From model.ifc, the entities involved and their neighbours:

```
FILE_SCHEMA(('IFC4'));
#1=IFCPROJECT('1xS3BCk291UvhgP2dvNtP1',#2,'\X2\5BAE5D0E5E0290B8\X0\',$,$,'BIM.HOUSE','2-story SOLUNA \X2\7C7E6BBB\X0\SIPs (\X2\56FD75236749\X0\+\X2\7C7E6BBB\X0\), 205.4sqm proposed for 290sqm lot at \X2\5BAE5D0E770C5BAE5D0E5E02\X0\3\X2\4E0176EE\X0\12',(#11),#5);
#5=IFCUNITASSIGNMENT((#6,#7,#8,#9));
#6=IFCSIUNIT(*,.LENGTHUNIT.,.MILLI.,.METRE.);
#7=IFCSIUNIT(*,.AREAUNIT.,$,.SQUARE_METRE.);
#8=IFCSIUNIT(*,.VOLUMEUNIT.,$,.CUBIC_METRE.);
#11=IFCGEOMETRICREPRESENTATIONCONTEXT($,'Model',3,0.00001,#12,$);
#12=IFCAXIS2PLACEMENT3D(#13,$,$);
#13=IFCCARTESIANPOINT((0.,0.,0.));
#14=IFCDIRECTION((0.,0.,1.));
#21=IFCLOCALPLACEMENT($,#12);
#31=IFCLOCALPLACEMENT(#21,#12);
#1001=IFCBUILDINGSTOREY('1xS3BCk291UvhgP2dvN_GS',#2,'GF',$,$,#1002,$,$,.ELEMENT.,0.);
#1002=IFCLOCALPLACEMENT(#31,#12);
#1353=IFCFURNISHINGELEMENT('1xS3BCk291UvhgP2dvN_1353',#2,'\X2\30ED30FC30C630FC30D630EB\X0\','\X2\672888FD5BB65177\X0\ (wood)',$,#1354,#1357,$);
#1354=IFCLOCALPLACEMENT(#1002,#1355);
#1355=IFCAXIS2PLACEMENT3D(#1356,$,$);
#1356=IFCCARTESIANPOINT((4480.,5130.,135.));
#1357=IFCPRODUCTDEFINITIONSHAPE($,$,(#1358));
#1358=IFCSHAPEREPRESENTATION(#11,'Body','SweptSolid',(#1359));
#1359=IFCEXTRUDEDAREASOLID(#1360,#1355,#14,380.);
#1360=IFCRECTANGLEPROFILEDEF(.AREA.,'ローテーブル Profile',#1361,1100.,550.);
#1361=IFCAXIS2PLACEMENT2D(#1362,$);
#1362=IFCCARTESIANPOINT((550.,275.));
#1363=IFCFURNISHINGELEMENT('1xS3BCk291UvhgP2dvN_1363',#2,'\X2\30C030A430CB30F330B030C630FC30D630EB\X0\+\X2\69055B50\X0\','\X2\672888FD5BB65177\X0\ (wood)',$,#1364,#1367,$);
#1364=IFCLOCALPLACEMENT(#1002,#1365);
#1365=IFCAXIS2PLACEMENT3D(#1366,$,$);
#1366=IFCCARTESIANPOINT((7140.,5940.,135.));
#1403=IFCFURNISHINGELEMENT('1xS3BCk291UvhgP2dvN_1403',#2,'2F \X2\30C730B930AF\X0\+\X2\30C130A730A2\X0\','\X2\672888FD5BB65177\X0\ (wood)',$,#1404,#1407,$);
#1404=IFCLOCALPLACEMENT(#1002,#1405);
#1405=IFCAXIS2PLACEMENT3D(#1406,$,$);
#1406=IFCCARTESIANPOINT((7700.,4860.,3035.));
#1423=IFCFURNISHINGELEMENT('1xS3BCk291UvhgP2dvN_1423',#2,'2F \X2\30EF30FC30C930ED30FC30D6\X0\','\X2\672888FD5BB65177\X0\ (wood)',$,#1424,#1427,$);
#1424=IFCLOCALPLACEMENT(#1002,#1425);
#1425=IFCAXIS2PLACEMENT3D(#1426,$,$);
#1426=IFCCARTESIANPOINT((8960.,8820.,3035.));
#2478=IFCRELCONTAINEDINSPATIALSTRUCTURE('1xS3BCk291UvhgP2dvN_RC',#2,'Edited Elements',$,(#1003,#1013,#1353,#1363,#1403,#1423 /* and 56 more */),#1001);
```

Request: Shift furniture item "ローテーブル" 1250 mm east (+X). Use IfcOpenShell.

```python
import ifcopenshell
import ifcopenshell.api.geometry
import ifcopenshell.util.placement
import ifcopenshell.util.unit

model = ifcopenshell.open("model.ifc")
unit_scale = ifcopenshell.util.unit.calculate_unit_scale(model)

item = model.by_guid("1xS3BCk291UvhgP2dvN_1353")
matrix = ifcopenshell.util.placement.get_local_placement(item.ObjectPlacement)
matrix[0, 3] += 1.25 / unit_scale
ifcopenshell.api.geometry.edit_object_placement(model, product=item, matrix=matrix, is_si=False)

print(ifcopenshell.util.placement.get_local_placement(item.ObjectPlacement).round(3) + 0.0)

model.write("model_v2.ifc")
```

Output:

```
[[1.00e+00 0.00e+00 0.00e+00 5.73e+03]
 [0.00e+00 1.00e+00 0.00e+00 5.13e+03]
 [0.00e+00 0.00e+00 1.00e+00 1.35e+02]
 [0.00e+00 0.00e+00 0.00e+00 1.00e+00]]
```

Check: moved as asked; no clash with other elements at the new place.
